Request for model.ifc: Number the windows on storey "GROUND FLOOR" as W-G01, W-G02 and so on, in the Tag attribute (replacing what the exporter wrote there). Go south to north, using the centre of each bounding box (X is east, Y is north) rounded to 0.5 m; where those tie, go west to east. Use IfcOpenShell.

First a look at what the model holds.

```python
import ifcopenshell
import ifcopenshell.util.element
import ifcopenshell.util.placement

model = ifcopenshell.open("model.ifc")
print(model.schema)
storey = next(s for s in model.by_type("IfcBuildingStorey") if s.Name == "GROUND FLOOR")
windows = [e for e in ifcopenshell.util.element.get_decomposition(storey) if e.is_a("IfcWindow")]
for e in sorted(windows, key=lambda e: e.id()):
    origin = ifcopenshell.util.placement.get_local_placement(e.ObjectPlacement)[:3, 3]
    print(e.id(), e.Tag, e.Name, origin.round(2) + 0.0, sep=" | ")
```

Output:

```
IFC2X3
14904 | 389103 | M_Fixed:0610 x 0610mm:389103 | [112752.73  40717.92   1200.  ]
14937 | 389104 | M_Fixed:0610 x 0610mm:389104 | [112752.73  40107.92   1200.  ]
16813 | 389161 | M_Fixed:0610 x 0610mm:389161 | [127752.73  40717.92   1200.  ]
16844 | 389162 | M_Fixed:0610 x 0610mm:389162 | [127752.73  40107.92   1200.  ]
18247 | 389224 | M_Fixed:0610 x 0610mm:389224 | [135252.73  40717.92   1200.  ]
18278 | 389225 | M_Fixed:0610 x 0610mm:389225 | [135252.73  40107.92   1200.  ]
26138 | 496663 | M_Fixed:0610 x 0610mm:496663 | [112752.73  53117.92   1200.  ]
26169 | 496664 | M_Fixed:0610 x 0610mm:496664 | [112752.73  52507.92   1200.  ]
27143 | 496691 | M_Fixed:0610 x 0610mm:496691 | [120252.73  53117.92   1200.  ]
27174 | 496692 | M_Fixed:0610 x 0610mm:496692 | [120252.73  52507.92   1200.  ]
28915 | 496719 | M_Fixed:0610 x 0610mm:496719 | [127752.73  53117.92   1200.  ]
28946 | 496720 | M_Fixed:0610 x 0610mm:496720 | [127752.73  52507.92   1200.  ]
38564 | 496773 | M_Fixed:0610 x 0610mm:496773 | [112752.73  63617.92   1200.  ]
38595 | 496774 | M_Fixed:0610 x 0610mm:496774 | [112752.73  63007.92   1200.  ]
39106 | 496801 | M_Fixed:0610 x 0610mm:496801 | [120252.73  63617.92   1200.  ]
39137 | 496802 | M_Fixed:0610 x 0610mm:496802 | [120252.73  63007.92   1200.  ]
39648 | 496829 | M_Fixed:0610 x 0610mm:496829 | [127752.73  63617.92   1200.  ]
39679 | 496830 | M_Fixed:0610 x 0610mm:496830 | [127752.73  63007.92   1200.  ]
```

```python
import ifcopenshell
import ifcopenshell.geom
import ifcopenshell.util.element
import ifcopenshell.util.shape

model = ifcopenshell.open("model.ifc")
settings = ifcopenshell.geom.settings()
settings.set("use-world-coords", True)


def centre(element):
    shape = ifcopenshell.geom.create_shape(settings, element)
    return ifcopenshell.util.shape.get_bbox_centroid(shape.geometry)


storey = next(s for s in model.by_type("IfcBuildingStorey") if s.Name == "GROUND FLOOR")
windows = [e for e in ifcopenshell.util.element.get_decomposition(storey) if e.is_a("IfcWindow")]

# Insertion points can sit at a corner or the storey origin, so sort by the geometry (in metres).
centres = {e: centre(e) for e in windows}
windows.sort(key=lambda e: (round(centres[e][1] / 0.5), centres[e][0]))

for i, e in enumerate(windows, start=1):
    number = f"W-G{i:02d}"
    e.Tag = number
    print(e.id(), number)

model.write("model_edited.ifc")
```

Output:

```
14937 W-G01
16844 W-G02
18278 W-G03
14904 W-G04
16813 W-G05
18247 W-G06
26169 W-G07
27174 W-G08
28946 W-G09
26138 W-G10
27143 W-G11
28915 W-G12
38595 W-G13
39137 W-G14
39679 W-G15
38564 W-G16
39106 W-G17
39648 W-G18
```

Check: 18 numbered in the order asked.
